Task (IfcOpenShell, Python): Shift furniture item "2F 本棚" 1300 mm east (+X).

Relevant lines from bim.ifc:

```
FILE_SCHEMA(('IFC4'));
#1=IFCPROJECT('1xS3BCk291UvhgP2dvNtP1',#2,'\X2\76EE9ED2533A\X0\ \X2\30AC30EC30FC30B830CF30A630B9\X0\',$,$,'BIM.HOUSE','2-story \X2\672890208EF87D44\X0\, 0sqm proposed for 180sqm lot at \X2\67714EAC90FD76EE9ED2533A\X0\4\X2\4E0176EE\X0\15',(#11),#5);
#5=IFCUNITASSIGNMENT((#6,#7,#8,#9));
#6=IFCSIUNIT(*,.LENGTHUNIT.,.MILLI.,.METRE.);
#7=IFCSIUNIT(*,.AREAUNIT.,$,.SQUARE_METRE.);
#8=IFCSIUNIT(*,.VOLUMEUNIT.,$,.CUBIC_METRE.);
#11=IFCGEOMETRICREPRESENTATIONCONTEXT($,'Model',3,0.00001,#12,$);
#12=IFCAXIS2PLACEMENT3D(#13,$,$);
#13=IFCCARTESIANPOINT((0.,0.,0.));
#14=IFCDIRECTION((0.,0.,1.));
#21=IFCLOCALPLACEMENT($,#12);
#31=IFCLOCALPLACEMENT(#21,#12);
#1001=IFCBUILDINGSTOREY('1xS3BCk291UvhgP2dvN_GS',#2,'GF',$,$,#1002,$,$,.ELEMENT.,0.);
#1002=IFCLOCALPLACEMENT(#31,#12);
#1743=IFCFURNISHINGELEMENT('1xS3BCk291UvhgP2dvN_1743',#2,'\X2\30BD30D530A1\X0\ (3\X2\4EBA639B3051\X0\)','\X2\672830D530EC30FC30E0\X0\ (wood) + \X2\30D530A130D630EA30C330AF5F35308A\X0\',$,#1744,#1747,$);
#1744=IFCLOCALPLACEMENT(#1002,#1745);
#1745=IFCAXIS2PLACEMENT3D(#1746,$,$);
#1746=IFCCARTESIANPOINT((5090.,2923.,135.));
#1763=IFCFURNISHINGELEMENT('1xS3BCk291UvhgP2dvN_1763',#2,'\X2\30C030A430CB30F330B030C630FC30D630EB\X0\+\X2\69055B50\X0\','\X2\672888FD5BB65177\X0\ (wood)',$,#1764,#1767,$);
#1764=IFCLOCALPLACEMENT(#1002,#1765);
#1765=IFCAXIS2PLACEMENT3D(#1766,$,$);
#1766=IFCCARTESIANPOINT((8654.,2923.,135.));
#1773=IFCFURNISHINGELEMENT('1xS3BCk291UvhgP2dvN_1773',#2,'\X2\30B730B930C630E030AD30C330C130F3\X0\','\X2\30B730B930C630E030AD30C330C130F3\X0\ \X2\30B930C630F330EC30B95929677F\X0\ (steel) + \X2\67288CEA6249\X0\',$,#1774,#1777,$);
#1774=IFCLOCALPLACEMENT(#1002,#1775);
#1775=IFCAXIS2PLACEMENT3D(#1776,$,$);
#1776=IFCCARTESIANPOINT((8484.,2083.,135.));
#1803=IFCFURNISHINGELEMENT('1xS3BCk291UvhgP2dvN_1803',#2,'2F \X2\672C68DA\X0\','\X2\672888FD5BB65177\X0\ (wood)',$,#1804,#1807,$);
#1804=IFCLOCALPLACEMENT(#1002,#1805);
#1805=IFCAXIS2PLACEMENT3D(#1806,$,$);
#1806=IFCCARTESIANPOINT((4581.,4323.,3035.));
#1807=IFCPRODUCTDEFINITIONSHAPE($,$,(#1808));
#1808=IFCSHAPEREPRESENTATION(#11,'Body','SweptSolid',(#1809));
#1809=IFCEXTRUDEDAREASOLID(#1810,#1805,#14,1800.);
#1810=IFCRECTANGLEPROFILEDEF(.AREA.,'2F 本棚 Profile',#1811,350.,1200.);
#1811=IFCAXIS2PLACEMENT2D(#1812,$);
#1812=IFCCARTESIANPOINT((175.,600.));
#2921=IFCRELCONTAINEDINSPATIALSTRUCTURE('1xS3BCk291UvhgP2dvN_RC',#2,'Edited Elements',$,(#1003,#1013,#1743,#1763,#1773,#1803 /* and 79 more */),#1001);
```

```python
import ifcopenshell
import ifcopenshell.api.geometry
import ifcopenshell.util.placement

model = ifcopenshell.open("bim.ifc")

item = model.by_id(1803)
matrix = ifcopenshell.util.placement.get_local_placement(item.ObjectPlacement)
matrix[0, 3] += 1300.0
ifcopenshell.api.geometry.edit_object_placement(model, product=item, matrix=matrix, is_si=False)

print(ifcopenshell.util.placement.get_local_placement(item.ObjectPlacement).round(3) + 0.0)

model.write("bim_edited.ifc")
```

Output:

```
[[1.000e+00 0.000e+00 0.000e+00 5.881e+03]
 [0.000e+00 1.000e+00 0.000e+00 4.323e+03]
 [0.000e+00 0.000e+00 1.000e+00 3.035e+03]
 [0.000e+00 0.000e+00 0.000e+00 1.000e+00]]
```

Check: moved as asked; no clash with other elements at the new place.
